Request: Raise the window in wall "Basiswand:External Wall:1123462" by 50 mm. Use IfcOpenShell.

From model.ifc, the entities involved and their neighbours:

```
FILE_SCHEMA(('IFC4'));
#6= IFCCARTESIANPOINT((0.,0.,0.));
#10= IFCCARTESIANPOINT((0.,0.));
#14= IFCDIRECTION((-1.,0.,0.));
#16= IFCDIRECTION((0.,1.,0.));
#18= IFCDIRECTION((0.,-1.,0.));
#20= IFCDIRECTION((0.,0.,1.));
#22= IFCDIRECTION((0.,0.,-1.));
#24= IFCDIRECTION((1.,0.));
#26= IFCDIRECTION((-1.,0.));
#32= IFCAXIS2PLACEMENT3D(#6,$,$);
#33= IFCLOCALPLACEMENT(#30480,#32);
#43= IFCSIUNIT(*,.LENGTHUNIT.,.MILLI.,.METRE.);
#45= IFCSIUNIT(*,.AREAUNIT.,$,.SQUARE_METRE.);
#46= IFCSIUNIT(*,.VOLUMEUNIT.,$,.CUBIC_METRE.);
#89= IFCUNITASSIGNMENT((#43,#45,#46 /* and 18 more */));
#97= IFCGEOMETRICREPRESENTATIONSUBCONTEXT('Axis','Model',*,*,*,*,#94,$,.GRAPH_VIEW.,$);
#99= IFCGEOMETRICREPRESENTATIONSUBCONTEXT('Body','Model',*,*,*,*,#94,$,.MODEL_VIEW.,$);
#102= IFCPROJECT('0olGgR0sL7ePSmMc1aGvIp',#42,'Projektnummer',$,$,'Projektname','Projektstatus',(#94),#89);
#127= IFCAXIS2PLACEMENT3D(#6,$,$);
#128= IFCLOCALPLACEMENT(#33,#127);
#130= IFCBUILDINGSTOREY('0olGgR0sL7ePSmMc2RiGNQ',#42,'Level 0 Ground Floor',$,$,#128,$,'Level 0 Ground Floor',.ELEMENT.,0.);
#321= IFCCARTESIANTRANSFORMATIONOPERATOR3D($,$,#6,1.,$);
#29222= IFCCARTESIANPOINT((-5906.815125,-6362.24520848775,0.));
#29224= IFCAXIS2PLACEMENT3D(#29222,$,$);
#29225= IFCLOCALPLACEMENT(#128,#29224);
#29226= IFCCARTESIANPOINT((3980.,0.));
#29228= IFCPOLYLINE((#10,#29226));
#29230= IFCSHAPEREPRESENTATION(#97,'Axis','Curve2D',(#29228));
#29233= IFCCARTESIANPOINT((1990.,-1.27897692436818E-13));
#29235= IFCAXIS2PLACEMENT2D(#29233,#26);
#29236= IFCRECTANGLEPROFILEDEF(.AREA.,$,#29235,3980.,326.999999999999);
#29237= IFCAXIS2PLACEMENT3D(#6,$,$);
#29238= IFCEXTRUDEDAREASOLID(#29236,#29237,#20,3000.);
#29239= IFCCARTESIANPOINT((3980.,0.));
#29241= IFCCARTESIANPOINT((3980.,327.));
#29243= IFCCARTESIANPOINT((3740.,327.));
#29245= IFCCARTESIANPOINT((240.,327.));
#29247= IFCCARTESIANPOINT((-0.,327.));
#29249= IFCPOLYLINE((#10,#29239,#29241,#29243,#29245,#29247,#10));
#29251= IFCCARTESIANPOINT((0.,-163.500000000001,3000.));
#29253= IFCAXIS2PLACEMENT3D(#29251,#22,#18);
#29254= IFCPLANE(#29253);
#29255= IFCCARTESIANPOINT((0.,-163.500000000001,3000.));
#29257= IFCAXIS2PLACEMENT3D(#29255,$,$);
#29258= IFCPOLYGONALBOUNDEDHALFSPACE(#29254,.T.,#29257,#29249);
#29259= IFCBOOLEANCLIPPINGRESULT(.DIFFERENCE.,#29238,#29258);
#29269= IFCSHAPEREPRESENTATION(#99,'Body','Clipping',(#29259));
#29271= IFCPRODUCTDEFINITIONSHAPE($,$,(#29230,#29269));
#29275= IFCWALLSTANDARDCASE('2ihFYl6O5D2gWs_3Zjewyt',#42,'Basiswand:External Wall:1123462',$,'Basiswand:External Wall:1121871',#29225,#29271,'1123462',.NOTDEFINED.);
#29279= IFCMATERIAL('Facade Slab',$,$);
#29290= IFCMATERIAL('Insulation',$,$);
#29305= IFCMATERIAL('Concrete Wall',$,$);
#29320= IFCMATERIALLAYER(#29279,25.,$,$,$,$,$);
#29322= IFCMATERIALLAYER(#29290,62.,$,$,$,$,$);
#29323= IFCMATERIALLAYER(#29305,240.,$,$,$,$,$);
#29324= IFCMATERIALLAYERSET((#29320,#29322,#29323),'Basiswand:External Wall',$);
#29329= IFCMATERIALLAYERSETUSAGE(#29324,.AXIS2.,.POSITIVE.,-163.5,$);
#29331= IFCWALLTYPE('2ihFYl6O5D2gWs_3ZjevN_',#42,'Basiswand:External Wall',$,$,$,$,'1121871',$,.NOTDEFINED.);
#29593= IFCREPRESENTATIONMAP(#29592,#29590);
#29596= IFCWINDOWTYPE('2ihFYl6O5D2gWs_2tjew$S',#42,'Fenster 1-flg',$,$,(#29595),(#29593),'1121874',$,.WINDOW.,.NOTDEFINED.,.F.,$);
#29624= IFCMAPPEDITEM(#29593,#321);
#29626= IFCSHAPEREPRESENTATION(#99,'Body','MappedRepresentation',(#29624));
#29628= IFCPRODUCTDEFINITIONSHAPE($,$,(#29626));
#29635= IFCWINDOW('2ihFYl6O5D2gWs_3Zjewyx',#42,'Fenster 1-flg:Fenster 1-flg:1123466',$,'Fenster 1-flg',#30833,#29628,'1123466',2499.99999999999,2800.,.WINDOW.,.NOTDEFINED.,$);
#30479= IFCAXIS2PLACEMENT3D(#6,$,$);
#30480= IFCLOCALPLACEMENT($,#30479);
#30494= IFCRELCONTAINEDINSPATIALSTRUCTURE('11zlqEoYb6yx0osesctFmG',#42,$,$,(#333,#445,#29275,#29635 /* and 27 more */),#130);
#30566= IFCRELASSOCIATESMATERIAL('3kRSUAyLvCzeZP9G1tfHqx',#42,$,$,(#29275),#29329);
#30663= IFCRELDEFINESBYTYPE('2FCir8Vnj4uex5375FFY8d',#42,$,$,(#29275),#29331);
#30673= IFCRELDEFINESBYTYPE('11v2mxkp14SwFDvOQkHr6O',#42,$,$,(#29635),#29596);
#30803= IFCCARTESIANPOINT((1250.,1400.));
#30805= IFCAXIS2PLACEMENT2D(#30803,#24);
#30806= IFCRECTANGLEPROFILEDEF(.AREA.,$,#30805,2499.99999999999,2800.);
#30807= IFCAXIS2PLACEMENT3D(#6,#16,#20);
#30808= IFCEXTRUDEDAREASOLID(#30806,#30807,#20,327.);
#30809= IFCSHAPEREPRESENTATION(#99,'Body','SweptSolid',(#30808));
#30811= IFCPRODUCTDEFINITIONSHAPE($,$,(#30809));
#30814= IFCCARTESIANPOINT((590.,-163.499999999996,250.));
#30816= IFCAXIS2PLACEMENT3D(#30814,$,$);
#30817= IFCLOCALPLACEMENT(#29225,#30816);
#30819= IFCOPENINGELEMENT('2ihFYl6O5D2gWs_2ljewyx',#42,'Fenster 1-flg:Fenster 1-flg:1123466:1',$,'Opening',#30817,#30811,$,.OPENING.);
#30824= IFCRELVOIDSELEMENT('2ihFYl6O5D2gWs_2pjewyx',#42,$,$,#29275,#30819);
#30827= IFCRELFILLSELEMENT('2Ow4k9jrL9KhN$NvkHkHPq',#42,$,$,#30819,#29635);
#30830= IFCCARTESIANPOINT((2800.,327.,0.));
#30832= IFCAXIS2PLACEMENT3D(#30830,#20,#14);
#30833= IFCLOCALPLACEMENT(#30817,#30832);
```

```python
import numpy as np
import ifcopenshell
import ifcopenshell.api.geometry
import ifcopenshell.util.placement
import ifcopenshell.util.unit

model = ifcopenshell.open("model.ifc")
unit_scale = ifcopenshell.util.unit.calculate_unit_scale(model)

window = model.by_guid("2ihFYl6O5D2gWs_3Zjewyx")
opening = window.FillsVoids[0].RelatingOpeningElement
dz = 50.0

shift = np.array([0.0, 0.0, dz])
# The window is placed relative to its opening, so it follows when the opening moves.
matrix = ifcopenshell.util.placement.get_local_placement(opening.ObjectPlacement)
matrix[:3, 3] += shift
ifcopenshell.api.geometry.edit_object_placement(
    model, product=opening, matrix=matrix, is_si=False, should_transform_children=True
)

print(f"moved by {dz * unit_scale:+.3f} m")

model.write("model_v2.ifc")
```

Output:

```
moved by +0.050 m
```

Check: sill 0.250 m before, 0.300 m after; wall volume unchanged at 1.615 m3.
